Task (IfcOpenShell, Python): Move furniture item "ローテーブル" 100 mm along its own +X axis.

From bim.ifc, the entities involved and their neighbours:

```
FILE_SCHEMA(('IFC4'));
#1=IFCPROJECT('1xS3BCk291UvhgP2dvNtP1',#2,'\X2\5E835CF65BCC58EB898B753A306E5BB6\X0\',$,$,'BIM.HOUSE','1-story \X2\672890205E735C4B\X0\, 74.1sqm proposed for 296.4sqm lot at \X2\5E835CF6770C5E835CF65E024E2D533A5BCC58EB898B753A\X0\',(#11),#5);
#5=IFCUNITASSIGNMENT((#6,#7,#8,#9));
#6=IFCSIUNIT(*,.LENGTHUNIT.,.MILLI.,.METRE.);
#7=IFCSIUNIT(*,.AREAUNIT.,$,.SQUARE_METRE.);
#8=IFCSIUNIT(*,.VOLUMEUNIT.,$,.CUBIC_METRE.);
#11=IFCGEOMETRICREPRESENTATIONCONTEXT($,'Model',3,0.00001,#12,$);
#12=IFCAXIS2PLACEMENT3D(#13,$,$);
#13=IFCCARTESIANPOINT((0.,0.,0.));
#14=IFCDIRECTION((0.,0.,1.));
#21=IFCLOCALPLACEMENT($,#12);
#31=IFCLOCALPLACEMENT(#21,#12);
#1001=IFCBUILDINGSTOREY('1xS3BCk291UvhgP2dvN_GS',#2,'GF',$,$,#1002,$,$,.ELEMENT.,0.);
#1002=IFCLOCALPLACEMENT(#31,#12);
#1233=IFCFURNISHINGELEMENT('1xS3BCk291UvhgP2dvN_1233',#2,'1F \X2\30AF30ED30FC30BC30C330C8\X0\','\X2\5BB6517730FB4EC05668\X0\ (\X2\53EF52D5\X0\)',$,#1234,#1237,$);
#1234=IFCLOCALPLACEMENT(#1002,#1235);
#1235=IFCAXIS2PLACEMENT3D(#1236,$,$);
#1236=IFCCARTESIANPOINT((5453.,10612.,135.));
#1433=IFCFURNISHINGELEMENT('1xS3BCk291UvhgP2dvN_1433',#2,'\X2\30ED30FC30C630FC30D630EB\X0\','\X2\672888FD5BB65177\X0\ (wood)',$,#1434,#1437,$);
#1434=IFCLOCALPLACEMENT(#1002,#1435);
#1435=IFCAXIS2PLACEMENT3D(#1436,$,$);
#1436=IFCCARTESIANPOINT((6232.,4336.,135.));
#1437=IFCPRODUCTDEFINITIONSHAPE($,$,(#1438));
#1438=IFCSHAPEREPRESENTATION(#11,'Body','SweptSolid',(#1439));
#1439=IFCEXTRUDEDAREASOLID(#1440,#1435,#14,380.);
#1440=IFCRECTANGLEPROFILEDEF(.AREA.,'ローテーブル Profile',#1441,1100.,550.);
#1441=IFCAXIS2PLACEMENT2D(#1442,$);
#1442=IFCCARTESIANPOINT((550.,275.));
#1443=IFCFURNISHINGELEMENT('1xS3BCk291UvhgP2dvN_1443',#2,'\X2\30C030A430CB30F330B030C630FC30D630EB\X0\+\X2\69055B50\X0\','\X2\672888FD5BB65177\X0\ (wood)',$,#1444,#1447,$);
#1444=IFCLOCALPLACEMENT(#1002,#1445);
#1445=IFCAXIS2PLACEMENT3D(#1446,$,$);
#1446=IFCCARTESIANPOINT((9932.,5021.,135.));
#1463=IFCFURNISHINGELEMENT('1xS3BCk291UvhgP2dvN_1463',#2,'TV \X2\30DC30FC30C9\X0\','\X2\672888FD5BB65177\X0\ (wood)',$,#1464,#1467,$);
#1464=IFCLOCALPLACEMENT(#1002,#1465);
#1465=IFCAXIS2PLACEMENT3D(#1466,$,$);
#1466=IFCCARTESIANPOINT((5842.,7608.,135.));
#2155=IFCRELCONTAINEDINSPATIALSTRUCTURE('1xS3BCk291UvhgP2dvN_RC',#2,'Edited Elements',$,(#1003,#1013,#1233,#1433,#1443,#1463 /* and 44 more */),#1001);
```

```python
import ifcopenshell
import ifcopenshell.api.geometry
import ifcopenshell.util.placement

model = ifcopenshell.open("bim.ifc")

item = model.by_guid("1xS3BCk291UvhgP2dvN_1433")
matrix = ifcopenshell.util.placement.get_local_placement(item.ObjectPlacement)
matrix[:3, 3] += matrix[:3, 0] * 100.0
ifcopenshell.api.geometry.edit_object_placement(model, product=item, matrix=matrix, is_si=False)

print(ifcopenshell.util.placement.get_local_placement(item.ObjectPlacement).round(3) + 0.0)

model.write("bim_v2.ifc")
```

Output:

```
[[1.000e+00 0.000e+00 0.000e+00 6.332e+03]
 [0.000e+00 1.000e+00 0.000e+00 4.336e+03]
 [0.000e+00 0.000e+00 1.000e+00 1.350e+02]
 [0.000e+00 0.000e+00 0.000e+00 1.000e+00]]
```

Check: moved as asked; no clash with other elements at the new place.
